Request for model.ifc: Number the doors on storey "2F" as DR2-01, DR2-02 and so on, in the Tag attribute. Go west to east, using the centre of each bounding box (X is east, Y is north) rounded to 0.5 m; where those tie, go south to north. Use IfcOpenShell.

First a look at what the model holds.

```python
import ifcopenshell
import ifcopenshell.util.element
import ifcopenshell.util.placement

model = ifcopenshell.open("model.ifc")
print(model.schema)
storey = next(s for s in model.by_type("IfcBuildingStorey") if s.Name == "2F")
doors = [e for e in ifcopenshell.util.element.get_decomposition(storey) if e.is_a("IfcDoor")]
for e in sorted(doors, key=lambda e: e.id()):
    origin = ifcopenshell.util.placement.get_local_placement(e.ObjectPlacement)[:3, 3]
    print(e.id(), e.Tag, e.Name, origin.round(2) + 0.0, sep=" | ")
```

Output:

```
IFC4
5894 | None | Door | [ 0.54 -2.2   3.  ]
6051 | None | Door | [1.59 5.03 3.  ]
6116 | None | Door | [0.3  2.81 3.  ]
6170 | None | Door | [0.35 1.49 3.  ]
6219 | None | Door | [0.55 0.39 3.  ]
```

```python
import ifcopenshell
import ifcopenshell.geom
import ifcopenshell.util.element
import ifcopenshell.util.shape

model = ifcopenshell.open("model.ifc")
settings = ifcopenshell.geom.settings()
settings.set("use-world-coords", True)


def centre(element):
    shape = ifcopenshell.geom.create_shape(settings, element)
    return ifcopenshell.util.shape.get_bbox_centroid(shape.geometry)


storey = next(s for s in model.by_type("IfcBuildingStorey") if s.Name == "2F")
doors = [e for e in ifcopenshell.util.element.get_decomposition(storey) if e.is_a("IfcDoor")]

# Insertion points can sit at a corner or the storey origin, so sort by the geometry (in metres).
centres = {e: centre(e) for e in doors}
doors.sort(key=lambda e: (round(centres[e][0] / 0.5), centres[e][1]))

for i, e in enumerate(doors, start=1):
    number = f"DR2-{i:02d}"
    e.Tag = number
    print(e.id(), number)

model.write("model_updated.ifc")
```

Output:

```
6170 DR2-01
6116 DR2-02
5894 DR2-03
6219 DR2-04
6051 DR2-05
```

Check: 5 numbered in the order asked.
